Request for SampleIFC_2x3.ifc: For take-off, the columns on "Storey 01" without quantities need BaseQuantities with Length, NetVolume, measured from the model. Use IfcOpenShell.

First a look at what the model holds.

```python
import ifcopenshell
import ifcopenshell.util.element
import ifcopenshell.util.unit

model = ifcopenshell.open("SampleIFC_2x3.ifc")
print(model.schema)
for unit_type in ("LENGTHUNIT", "AREAUNIT", "VOLUMEUNIT"):
    print(unit_type, ifcopenshell.util.unit.calculate_unit_scale(model, unit_type))
storey = next(s for s in model.by_type("IfcBuildingStorey") if s.Name == "Storey 01")
columns = [e for e in ifcopenshell.util.element.get_decomposition(storey) if e.is_a("IfcColumn")]
for e in sorted(columns, key=lambda e: e.id()):
    print(e.id(), e.is_a(), e.Name, list(ifcopenshell.util.element.get_psets(e, qtos_only=True)), sep=" | ")
```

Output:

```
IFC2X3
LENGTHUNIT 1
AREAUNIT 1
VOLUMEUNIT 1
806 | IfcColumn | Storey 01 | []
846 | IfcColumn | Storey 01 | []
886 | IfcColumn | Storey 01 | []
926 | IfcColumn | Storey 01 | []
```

```python
import ifcopenshell
import ifcopenshell.api.pset
import ifcopenshell.geom
import ifcopenshell.util.element
import ifcopenshell.util.shape
import ifcopenshell.util.unit

model = ifcopenshell.open("SampleIFC_2x3.ifc")
unit_scale = ifcopenshell.util.unit.calculate_unit_scale(model)
volume_scale = ifcopenshell.util.unit.calculate_unit_scale(model, "VOLUMEUNIT")
settings = ifcopenshell.geom.settings()

storey = next(s for s in model.by_type("IfcBuildingStorey") if s.Name == "Storey 01")
columns = [e for e in ifcopenshell.util.element.get_decomposition(storey) if e.is_a("IfcColumn")]

for e in sorted(columns, key=lambda e: e.id()):
    if ifcopenshell.util.element.get_psets(e, qtos_only=True, should_inherit=False):
        continue
    # Geometry comes back in metres, in the element's own axes.
    shape = ifcopenshell.geom.create_shape(settings, e)
    values = {
        "Length": ifcopenshell.util.shape.get_z(shape.geometry) / unit_scale,
        "NetVolume": ifcopenshell.util.shape.get_volume(shape.geometry) / volume_scale,
    }
    qto = ifcopenshell.api.pset.add_qto(model, product=e, name="BaseQuantities")
    ifcopenshell.api.pset.edit_qto(model, qto=qto, properties=values)
    print(e.id(), {k: round(v, 3) for k, v in values.items()})

model.write("SampleIFC_2x3_rev.ifc")
```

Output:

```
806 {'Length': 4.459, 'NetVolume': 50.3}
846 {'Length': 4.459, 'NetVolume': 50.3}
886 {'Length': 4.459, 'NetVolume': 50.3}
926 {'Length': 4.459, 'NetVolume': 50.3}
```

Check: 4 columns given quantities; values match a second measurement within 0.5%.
